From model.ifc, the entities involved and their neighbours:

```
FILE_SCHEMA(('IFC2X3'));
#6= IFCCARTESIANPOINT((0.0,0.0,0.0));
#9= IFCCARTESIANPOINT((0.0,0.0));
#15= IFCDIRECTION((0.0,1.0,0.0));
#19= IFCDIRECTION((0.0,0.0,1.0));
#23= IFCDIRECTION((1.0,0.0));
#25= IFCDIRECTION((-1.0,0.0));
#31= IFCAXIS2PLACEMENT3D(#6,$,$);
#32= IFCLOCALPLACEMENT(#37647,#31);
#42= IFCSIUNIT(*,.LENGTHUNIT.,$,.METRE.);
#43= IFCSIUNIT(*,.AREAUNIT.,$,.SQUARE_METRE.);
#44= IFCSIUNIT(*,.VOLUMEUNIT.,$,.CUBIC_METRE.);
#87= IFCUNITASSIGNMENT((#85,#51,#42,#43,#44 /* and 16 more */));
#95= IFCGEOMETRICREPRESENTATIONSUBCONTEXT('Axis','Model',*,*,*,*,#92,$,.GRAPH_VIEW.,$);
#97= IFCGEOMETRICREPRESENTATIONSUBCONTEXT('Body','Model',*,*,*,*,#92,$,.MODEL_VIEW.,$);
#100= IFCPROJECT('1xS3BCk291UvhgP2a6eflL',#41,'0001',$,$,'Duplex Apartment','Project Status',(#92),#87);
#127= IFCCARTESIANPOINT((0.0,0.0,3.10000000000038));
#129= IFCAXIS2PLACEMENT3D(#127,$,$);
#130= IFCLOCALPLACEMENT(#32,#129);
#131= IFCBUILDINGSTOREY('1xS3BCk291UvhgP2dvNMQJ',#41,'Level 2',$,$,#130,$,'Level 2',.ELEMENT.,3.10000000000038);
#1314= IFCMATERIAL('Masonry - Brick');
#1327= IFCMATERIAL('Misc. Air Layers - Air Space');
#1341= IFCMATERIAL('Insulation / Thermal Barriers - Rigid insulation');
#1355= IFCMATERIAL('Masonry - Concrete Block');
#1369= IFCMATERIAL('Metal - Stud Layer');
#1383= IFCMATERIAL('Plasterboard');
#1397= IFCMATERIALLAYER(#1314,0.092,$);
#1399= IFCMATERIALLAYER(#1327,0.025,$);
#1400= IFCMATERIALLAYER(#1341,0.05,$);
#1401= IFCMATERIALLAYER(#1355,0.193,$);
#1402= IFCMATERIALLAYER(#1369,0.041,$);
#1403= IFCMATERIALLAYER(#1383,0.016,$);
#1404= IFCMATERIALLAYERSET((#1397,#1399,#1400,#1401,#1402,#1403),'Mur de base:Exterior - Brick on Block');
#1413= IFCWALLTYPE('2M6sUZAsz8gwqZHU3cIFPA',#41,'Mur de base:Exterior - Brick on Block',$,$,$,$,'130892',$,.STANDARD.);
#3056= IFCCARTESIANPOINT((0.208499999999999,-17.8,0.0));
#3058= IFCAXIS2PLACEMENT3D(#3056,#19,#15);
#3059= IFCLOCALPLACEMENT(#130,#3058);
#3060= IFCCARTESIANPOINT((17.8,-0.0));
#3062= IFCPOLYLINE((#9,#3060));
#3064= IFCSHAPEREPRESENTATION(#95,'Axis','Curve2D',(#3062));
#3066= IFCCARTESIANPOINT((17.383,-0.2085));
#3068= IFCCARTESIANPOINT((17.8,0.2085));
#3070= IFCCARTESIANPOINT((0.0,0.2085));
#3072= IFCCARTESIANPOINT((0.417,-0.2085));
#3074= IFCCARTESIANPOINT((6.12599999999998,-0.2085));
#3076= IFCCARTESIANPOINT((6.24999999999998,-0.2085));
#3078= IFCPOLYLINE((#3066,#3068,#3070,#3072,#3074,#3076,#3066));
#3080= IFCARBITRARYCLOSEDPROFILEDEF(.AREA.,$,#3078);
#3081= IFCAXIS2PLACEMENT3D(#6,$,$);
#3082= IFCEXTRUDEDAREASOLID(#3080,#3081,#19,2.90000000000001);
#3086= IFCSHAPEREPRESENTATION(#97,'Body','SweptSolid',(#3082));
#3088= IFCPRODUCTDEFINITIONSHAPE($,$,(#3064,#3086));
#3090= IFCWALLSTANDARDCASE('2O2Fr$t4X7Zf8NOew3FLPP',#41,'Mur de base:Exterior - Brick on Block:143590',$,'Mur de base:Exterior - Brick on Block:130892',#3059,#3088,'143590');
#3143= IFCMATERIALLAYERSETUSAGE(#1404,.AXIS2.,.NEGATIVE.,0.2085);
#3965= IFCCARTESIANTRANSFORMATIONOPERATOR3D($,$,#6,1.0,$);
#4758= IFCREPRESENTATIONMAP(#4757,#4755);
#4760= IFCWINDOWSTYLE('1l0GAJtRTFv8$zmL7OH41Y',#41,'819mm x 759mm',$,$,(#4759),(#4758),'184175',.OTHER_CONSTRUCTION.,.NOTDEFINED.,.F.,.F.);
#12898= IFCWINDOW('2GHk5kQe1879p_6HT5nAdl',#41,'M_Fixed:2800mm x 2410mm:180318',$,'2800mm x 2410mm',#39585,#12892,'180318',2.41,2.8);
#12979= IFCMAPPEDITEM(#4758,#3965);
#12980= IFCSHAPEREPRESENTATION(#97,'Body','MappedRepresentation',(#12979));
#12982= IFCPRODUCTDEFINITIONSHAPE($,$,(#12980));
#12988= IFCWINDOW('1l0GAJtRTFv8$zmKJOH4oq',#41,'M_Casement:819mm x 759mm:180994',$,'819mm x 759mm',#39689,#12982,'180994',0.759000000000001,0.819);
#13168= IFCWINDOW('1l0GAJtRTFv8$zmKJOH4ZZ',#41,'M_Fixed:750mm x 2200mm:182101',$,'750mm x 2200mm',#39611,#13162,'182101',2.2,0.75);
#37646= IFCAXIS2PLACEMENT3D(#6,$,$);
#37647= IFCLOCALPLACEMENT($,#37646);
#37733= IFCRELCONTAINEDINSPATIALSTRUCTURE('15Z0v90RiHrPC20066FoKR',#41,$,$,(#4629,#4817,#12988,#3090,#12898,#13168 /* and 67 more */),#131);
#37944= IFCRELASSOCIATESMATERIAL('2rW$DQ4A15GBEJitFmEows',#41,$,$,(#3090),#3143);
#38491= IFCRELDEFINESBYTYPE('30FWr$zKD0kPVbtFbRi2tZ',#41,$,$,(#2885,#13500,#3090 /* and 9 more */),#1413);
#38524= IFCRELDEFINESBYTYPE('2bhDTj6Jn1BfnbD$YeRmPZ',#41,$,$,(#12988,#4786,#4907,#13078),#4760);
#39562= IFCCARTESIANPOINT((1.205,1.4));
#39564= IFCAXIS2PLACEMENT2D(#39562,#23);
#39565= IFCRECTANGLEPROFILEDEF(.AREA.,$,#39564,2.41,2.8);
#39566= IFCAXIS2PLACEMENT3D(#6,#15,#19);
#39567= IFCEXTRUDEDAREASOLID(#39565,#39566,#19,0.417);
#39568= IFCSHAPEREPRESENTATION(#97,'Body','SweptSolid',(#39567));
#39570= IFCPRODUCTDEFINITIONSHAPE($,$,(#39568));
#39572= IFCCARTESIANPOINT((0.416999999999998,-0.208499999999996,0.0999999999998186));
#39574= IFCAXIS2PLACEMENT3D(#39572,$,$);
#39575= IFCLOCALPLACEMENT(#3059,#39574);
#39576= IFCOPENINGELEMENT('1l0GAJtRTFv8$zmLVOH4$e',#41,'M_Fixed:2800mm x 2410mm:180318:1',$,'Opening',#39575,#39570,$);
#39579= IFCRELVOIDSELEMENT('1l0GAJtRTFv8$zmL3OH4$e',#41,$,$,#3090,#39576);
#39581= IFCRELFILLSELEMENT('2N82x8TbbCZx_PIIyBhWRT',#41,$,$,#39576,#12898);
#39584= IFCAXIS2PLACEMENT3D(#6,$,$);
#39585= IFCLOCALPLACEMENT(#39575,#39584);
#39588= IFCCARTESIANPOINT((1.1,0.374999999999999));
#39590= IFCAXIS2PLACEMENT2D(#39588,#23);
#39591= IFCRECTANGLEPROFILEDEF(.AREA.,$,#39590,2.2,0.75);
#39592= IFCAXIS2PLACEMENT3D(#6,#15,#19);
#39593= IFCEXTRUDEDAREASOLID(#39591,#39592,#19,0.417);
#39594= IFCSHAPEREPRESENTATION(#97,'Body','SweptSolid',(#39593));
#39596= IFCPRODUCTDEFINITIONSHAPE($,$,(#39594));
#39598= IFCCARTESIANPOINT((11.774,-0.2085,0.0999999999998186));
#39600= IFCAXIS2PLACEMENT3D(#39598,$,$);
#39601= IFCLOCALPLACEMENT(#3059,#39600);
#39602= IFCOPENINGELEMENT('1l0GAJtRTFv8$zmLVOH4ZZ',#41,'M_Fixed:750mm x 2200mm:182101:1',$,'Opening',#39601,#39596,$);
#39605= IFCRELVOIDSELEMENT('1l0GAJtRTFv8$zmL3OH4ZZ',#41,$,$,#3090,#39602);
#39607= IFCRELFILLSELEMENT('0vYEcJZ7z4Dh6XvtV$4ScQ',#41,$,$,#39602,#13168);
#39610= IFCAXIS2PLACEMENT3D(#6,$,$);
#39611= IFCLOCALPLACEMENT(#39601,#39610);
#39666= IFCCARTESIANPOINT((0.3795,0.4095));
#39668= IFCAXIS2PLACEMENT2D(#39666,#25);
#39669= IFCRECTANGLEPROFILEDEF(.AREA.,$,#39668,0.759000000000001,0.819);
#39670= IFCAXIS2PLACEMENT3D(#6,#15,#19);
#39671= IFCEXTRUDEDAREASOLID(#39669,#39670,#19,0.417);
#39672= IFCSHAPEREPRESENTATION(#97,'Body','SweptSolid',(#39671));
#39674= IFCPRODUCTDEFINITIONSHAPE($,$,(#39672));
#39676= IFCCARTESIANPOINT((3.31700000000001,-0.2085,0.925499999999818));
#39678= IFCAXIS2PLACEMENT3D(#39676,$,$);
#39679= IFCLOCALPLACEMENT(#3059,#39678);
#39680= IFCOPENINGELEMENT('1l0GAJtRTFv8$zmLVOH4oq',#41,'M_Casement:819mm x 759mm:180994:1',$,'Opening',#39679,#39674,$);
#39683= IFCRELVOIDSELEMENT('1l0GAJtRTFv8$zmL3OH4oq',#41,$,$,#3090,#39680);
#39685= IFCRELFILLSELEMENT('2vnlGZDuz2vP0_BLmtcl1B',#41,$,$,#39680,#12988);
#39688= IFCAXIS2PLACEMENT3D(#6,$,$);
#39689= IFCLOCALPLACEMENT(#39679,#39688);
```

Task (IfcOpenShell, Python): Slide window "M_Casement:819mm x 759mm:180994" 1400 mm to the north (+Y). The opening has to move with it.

```python
import ifcopenshell
import ifcopenshell.api.geometry
import ifcopenshell.util.placement
import ifcopenshell.util.unit

model = ifcopenshell.open("model.ifc")
unit_scale = ifcopenshell.util.unit.calculate_unit_scale(model)

window = model.by_guid("1l0GAJtRTFv8$zmKJOH4oq")
opening = window.FillsVoids[0].RelatingOpeningElement
wall = opening.VoidsElements[0].RelatingBuildingElement

wall_matrix = ifcopenshell.util.placement.get_local_placement(wall.ObjectPlacement)
shift = wall_matrix[:3, 0] * 1.4 / unit_scale
before = ifcopenshell.util.placement.get_local_placement(window.ObjectPlacement)[:3, 3].copy()

# The window is placed relative to its opening, so it follows when the opening moves.
matrix = ifcopenshell.util.placement.get_local_placement(opening.ObjectPlacement)
matrix[:3, 3] += shift
ifcopenshell.api.geometry.edit_object_placement(
    model, product=opening, matrix=matrix, is_si=False, should_transform_children=True
)

after = ifcopenshell.util.placement.get_local_placement(window.ObjectPlacement)[:3, 3]
print("window moved by", (after - before).round(3) + 0.0)

model.write("model_v2.ifc")
```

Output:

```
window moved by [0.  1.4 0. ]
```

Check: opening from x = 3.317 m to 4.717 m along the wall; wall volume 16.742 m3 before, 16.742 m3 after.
